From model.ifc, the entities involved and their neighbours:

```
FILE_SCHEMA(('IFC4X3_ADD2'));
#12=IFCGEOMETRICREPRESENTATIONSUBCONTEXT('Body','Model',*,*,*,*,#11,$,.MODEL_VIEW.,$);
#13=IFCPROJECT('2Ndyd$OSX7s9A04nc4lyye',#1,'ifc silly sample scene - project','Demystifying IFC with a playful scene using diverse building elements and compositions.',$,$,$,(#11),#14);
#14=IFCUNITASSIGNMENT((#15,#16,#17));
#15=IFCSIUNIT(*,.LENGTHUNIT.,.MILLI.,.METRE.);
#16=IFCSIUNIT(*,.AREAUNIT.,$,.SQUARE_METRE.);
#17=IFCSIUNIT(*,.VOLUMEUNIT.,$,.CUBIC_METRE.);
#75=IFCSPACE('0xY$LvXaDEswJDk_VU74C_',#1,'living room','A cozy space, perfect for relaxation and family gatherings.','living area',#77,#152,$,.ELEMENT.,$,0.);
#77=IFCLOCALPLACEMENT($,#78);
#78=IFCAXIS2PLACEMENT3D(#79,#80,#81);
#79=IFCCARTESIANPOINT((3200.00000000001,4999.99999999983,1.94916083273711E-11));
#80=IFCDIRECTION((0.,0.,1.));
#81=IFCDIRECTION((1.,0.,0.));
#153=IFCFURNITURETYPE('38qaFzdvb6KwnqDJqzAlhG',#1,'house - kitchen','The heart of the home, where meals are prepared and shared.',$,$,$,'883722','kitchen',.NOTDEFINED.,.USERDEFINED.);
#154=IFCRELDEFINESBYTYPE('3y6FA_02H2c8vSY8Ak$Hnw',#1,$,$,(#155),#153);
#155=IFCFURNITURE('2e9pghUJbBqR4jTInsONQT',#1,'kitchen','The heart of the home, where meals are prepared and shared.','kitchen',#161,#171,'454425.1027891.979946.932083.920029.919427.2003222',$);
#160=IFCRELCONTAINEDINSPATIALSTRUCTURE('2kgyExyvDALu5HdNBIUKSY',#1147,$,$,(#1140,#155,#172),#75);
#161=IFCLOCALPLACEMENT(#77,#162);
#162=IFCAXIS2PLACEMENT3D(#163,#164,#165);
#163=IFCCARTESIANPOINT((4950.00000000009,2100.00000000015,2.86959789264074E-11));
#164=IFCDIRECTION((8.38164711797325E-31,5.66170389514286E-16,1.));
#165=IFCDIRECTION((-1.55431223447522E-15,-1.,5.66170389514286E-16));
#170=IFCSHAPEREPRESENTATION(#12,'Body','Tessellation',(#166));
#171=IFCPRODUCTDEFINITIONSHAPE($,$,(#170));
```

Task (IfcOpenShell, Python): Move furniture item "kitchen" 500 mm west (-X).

```python
import ifcopenshell
import ifcopenshell.api.geometry
import ifcopenshell.util.placement

model = ifcopenshell.open("model.ifc")

item = model.by_guid("2e9pghUJbBqR4jTInsONQT")
matrix = ifcopenshell.util.placement.get_local_placement(item.ObjectPlacement)
matrix[0, 3] -= 500.0
ifcopenshell.api.geometry.edit_object_placement(model, product=item, matrix=matrix, is_si=False)

print(ifcopenshell.util.placement.get_local_placement(item.ObjectPlacement).round(3) + 0.0)

model.write("model_edited.ifc")
```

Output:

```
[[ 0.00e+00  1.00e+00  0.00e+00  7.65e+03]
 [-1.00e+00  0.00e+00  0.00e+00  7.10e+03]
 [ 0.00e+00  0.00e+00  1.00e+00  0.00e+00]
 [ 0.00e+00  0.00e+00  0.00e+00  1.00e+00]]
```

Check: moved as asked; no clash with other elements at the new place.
